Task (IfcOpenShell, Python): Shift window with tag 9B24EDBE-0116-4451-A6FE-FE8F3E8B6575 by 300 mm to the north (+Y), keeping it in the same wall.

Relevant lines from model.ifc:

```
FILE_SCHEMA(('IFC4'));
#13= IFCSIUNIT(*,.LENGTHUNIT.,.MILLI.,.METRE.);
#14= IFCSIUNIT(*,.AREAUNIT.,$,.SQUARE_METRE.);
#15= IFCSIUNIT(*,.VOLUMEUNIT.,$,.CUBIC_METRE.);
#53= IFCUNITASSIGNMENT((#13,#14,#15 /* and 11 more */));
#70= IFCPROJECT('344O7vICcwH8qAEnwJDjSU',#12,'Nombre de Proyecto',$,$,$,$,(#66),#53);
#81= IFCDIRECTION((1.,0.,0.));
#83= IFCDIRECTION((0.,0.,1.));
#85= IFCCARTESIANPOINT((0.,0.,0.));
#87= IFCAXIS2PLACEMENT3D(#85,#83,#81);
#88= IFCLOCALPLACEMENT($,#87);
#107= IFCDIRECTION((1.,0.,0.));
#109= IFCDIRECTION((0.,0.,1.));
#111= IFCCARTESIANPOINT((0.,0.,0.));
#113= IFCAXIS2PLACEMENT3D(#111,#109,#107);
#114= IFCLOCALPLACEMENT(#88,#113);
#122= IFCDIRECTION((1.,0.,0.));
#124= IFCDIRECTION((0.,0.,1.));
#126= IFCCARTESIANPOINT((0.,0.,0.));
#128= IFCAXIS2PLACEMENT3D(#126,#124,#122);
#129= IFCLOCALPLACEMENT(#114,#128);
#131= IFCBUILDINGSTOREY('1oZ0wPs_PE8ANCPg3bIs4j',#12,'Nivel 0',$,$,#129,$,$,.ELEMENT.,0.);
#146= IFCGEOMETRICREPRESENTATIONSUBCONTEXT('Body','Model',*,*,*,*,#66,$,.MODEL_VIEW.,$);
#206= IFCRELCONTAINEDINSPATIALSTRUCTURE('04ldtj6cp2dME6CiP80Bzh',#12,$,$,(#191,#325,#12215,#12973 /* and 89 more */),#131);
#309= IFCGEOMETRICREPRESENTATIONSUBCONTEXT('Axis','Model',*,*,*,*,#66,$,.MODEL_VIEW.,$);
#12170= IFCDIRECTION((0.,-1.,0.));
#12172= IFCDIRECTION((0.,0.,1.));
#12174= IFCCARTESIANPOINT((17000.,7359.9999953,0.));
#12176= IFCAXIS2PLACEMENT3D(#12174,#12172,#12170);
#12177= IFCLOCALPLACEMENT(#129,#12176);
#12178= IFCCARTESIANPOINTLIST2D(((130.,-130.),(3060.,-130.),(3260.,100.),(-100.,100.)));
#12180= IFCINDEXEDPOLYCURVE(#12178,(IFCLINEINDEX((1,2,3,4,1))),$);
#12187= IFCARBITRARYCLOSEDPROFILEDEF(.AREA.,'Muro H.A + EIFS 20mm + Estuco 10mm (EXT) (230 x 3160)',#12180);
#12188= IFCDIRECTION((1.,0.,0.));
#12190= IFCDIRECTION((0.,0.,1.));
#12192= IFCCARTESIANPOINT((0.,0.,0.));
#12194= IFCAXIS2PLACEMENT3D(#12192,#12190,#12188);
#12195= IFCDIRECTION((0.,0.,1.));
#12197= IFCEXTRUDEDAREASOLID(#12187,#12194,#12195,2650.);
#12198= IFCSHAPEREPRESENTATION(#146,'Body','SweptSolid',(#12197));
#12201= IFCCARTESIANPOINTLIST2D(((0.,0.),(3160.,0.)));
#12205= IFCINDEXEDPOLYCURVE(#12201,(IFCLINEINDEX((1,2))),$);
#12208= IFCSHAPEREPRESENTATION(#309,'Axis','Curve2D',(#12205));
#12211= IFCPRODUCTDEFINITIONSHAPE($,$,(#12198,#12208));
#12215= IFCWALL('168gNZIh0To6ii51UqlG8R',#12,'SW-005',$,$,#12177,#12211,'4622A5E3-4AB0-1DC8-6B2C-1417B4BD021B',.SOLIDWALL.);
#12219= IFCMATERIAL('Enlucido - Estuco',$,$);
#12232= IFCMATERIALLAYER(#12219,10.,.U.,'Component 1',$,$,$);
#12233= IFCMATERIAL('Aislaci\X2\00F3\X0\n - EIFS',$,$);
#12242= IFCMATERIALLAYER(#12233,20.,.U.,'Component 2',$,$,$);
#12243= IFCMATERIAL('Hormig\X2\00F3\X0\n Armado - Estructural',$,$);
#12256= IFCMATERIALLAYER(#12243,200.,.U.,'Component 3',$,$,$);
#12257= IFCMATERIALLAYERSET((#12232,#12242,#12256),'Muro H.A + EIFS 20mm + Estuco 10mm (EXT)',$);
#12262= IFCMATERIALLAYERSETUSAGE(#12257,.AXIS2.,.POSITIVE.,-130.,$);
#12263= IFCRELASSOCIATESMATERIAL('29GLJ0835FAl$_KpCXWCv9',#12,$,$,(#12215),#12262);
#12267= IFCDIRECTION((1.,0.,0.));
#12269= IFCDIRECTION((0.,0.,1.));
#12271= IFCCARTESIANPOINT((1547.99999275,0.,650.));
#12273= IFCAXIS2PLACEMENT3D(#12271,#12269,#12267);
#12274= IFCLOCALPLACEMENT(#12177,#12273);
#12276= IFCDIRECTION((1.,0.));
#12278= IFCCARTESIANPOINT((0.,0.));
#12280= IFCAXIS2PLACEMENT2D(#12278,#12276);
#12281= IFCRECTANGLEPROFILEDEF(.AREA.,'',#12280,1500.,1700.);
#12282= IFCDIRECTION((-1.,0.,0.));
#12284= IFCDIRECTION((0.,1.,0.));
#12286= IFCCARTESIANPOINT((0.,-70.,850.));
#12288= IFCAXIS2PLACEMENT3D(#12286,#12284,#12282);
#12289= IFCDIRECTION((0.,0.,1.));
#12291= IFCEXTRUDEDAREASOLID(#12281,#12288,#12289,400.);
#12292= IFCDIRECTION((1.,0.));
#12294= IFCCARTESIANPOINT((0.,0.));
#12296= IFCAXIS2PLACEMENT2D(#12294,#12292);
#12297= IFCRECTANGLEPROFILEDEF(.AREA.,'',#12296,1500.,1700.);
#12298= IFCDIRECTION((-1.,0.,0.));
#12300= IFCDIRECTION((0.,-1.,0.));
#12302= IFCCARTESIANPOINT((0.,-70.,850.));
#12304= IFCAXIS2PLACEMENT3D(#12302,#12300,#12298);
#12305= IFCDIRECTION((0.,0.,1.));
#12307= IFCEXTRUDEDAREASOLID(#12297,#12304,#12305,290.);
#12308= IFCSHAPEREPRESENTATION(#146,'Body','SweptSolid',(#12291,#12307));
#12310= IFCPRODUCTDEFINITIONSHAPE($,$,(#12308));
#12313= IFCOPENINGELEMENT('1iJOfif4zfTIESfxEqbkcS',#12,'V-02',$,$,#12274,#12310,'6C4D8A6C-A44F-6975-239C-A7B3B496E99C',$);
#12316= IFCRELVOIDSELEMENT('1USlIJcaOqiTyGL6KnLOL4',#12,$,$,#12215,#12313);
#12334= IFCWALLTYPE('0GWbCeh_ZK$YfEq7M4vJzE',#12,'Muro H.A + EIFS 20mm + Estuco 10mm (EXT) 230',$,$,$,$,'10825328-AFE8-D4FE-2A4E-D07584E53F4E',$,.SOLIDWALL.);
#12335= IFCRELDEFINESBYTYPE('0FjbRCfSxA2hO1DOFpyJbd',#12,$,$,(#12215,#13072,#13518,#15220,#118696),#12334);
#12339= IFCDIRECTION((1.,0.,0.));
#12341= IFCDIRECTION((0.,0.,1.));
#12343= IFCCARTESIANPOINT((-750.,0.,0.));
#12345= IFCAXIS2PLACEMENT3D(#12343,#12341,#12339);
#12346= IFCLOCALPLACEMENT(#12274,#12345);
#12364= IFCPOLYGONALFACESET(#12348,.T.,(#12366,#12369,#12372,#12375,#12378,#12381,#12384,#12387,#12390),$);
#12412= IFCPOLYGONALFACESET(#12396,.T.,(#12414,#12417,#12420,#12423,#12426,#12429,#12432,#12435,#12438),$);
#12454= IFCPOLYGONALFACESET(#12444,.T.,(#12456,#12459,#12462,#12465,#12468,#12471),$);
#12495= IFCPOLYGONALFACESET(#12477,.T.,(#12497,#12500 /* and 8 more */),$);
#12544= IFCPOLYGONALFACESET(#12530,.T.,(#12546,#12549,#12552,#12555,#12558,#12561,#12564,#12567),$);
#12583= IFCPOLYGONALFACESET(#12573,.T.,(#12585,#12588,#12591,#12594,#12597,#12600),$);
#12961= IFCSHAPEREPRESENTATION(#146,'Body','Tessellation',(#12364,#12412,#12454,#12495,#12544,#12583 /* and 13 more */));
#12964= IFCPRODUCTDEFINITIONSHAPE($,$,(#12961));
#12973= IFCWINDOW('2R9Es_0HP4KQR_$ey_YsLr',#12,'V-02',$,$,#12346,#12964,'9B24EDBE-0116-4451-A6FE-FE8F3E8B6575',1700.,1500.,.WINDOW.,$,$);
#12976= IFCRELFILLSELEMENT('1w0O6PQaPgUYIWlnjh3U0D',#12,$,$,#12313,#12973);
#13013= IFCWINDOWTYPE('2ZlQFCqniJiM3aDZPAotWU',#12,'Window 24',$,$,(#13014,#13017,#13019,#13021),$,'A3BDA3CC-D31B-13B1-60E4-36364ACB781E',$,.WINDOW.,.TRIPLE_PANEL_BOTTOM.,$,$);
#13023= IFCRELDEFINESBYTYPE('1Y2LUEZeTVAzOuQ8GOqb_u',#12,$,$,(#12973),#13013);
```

```python
import ifcopenshell
import ifcopenshell.api.geometry
import ifcopenshell.util.placement
import ifcopenshell.util.unit

model = ifcopenshell.open("model.ifc")
unit_scale = ifcopenshell.util.unit.calculate_unit_scale(model)

window = model.by_id(12973)
opening = window.FillsVoids[0].RelatingOpeningElement
wall = opening.VoidsElements[0].RelatingBuildingElement

wall_matrix = ifcopenshell.util.placement.get_local_placement(wall.ObjectPlacement)
shift = wall_matrix[:3, 0] * -0.3 / unit_scale
before = ifcopenshell.util.placement.get_local_placement(window.ObjectPlacement)[:3, 3].copy()

# The window is placed relative to its opening, so it follows when the opening moves.
matrix = ifcopenshell.util.placement.get_local_placement(opening.ObjectPlacement)
matrix[:3, 3] += shift
ifcopenshell.api.geometry.edit_object_placement(
    model, product=opening, matrix=matrix, is_si=False, should_transform_children=True
)

after = ifcopenshell.util.placement.get_local_placement(window.ObjectPlacement)[:3, 3]
print("window moved by", (after - before).round(3) + 0.0)

model.write("model_updated.ifc")
```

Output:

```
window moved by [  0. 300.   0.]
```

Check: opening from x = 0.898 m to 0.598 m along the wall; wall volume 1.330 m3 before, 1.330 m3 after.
